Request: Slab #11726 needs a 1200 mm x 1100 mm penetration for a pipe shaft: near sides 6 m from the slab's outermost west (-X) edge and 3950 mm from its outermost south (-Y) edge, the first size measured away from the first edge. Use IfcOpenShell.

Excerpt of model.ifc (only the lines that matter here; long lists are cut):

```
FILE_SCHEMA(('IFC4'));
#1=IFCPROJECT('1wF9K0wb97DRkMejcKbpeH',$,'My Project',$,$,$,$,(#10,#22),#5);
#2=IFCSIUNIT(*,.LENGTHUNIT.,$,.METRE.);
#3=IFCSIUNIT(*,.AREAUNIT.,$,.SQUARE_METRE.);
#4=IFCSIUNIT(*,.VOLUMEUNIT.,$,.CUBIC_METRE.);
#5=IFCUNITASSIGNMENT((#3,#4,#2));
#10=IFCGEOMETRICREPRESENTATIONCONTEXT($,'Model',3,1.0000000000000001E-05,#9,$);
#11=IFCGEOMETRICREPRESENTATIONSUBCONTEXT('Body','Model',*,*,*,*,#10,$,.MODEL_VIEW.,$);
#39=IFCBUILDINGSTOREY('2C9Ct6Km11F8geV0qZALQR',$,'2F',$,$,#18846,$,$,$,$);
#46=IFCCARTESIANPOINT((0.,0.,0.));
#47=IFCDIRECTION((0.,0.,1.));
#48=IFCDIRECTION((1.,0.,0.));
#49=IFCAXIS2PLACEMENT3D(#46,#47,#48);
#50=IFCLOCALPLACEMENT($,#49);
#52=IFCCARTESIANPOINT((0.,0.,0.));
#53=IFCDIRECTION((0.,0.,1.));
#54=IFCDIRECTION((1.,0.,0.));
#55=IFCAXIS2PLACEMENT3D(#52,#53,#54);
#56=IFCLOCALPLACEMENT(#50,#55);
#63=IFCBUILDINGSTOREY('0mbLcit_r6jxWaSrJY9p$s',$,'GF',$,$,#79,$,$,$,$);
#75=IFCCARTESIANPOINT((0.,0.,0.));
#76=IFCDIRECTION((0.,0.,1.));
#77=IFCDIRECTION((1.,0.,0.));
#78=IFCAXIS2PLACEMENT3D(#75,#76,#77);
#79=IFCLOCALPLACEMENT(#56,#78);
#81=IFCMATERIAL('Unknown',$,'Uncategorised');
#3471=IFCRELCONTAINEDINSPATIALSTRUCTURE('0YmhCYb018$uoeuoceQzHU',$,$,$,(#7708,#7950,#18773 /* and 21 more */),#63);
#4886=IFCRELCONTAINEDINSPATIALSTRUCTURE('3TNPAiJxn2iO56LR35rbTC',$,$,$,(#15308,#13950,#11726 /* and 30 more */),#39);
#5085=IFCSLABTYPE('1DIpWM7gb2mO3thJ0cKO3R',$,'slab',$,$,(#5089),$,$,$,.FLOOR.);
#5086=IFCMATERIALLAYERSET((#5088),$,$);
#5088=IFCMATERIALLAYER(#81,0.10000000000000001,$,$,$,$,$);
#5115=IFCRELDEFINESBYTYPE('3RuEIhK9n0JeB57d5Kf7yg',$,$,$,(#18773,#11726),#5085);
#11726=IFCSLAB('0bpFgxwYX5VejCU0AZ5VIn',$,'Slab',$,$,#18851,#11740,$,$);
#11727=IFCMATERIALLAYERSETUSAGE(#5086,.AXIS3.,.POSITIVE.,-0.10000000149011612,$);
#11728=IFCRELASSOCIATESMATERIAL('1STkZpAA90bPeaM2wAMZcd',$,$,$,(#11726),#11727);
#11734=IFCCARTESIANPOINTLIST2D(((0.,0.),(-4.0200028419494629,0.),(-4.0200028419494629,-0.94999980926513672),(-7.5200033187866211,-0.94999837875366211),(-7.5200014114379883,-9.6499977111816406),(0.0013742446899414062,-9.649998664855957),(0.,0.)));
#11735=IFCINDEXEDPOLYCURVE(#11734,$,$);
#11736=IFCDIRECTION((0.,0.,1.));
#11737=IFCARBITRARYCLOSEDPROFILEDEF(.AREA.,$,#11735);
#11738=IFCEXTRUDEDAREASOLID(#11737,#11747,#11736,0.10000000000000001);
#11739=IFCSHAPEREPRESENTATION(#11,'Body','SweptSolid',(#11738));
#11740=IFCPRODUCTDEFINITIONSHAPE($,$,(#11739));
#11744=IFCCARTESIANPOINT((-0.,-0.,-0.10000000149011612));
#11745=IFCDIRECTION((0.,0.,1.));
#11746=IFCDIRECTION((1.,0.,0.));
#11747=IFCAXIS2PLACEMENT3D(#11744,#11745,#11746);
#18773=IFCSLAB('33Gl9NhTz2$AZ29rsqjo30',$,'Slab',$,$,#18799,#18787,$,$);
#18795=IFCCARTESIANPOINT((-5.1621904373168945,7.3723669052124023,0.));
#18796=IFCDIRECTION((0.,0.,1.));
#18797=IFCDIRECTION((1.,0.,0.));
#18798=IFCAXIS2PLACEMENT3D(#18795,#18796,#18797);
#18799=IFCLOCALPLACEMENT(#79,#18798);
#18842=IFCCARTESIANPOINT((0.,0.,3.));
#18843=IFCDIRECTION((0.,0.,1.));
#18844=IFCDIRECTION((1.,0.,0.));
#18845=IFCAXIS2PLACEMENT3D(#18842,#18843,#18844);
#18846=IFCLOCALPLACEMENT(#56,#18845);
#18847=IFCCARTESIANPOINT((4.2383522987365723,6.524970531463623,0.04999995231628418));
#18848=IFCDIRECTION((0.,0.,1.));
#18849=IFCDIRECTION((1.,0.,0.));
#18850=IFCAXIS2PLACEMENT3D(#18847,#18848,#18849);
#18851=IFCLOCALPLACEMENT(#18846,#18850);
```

```python
import numpy as np
import ifcopenshell
import ifcopenshell.api.feature
import ifcopenshell.api.geometry
import ifcopenshell.api.root
import ifcopenshell.geom
import ifcopenshell.util.placement
import ifcopenshell.util.representation
import ifcopenshell.util.shape
import ifcopenshell.util.unit

model = ifcopenshell.open("model.ifc")
unit_scale = ifcopenshell.util.unit.calculate_unit_scale(model)
settings = ifcopenshell.geom.settings()


def volume(element):
    """Net volume in cubic metres, openings subtracted."""
    shape = ifcopenshell.geom.create_shape(settings, element)
    return ifcopenshell.util.shape.get_volume(shape.geometry)


slab = model.by_guid("0bpFgxwYX5VejCU0AZ5VIn")
before = volume(slab)

# Extent in the slab's own axes, in metres. The edges named are its -X and -Y sides.
slab_shape = ifcopenshell.geom.create_shape(settings, slab)
vertices = ifcopenshell.util.shape.get_vertices(slab_shape.geometry)
x_min, y_min, bottom = vertices.min(axis=0)
top = vertices[:, 2].max()

opening = ifcopenshell.api.root.create_entity(model, ifc_class="IfcOpeningElement", name="Pipe shaft opening", predefined_type="OPENING")
context = ifcopenshell.util.representation.get_context(model, "Model", "Body", "MODEL_VIEW")
width, depth = 1.2, 1.1
outline = [(0.0, 0.0), (width, 0.0), (width, depth), (0.0, depth), (0.0, 0.0)]
# Overshoot both faces by 50 mm so the cut is clean.
shape = ifcopenshell.api.geometry.add_slab_representation(
    model, context=context, depth=top - bottom + 0.1, polyline=outline
)
ifcopenshell.api.geometry.assign_representation(model, product=opening, representation=shape)

matrix = ifcopenshell.util.placement.get_local_placement(slab.ObjectPlacement)
matrix[:, 3] = matrix @ np.append(np.array([x_min + 6, y_min + 3.95, bottom - 0.05]) / unit_scale, 1.0)
ifcopenshell.api.geometry.edit_object_placement(model, product=opening, matrix=matrix, is_si=False)
ifcopenshell.api.feature.add_feature(model, feature=opening, element=slab)

after = volume(slab)

print(f"slab volume {before:.3f} -> {after:.3f} m3")

model.write("model_updated.ifc")
```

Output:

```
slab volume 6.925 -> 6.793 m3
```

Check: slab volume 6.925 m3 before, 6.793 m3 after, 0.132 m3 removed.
